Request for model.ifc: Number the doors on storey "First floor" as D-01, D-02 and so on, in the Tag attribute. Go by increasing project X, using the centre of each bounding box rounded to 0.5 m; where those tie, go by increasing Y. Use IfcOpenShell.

First a look at what the model holds.

```python
import ifcopenshell
import ifcopenshell.util.element
import ifcopenshell.util.placement

model = ifcopenshell.open("model.ifc")
print(model.schema)
storey = next(s for s in model.by_type("IfcBuildingStorey") if s.Name == "First floor")
doors = [e for e in ifcopenshell.util.element.get_decomposition(storey) if e.is_a("IfcDoor")]
for e in sorted(doors, key=lambda e: e.id()):
    origin = ifcopenshell.util.placement.get_local_placement(e.ObjectPlacement)[:3, 3]
    print(e.id(), e.Tag, e.Name, origin.round(2) + 0.0, sep=" | ")
```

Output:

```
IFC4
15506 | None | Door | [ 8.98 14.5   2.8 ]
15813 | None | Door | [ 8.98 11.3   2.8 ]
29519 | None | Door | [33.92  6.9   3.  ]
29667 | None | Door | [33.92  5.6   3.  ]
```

```python
import ifcopenshell
import ifcopenshell.geom
import ifcopenshell.util.element
import ifcopenshell.util.shape

model = ifcopenshell.open("model.ifc")
settings = ifcopenshell.geom.settings()
settings.set("use-world-coords", True)


def centre(element):
    shape = ifcopenshell.geom.create_shape(settings, element)
    return ifcopenshell.util.shape.get_bbox_centroid(shape.geometry)


storey = next(s for s in model.by_type("IfcBuildingStorey") if s.Name == "First floor")
doors = [e for e in ifcopenshell.util.element.get_decomposition(storey) if e.is_a("IfcDoor")]

# Insertion points can sit at a corner or the storey origin, so sort by the geometry (in metres).
centres = {e: centre(e) for e in doors}
doors.sort(key=lambda e: (round(centres[e][0] / 0.5), centres[e][1]))

for i, e in enumerate(doors, start=1):
    number = f"D-{i:02d}"
    e.Tag = number
    print(e.id(), number)

model.write("model_updated.ifc")
```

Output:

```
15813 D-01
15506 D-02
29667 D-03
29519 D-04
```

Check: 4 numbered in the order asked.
